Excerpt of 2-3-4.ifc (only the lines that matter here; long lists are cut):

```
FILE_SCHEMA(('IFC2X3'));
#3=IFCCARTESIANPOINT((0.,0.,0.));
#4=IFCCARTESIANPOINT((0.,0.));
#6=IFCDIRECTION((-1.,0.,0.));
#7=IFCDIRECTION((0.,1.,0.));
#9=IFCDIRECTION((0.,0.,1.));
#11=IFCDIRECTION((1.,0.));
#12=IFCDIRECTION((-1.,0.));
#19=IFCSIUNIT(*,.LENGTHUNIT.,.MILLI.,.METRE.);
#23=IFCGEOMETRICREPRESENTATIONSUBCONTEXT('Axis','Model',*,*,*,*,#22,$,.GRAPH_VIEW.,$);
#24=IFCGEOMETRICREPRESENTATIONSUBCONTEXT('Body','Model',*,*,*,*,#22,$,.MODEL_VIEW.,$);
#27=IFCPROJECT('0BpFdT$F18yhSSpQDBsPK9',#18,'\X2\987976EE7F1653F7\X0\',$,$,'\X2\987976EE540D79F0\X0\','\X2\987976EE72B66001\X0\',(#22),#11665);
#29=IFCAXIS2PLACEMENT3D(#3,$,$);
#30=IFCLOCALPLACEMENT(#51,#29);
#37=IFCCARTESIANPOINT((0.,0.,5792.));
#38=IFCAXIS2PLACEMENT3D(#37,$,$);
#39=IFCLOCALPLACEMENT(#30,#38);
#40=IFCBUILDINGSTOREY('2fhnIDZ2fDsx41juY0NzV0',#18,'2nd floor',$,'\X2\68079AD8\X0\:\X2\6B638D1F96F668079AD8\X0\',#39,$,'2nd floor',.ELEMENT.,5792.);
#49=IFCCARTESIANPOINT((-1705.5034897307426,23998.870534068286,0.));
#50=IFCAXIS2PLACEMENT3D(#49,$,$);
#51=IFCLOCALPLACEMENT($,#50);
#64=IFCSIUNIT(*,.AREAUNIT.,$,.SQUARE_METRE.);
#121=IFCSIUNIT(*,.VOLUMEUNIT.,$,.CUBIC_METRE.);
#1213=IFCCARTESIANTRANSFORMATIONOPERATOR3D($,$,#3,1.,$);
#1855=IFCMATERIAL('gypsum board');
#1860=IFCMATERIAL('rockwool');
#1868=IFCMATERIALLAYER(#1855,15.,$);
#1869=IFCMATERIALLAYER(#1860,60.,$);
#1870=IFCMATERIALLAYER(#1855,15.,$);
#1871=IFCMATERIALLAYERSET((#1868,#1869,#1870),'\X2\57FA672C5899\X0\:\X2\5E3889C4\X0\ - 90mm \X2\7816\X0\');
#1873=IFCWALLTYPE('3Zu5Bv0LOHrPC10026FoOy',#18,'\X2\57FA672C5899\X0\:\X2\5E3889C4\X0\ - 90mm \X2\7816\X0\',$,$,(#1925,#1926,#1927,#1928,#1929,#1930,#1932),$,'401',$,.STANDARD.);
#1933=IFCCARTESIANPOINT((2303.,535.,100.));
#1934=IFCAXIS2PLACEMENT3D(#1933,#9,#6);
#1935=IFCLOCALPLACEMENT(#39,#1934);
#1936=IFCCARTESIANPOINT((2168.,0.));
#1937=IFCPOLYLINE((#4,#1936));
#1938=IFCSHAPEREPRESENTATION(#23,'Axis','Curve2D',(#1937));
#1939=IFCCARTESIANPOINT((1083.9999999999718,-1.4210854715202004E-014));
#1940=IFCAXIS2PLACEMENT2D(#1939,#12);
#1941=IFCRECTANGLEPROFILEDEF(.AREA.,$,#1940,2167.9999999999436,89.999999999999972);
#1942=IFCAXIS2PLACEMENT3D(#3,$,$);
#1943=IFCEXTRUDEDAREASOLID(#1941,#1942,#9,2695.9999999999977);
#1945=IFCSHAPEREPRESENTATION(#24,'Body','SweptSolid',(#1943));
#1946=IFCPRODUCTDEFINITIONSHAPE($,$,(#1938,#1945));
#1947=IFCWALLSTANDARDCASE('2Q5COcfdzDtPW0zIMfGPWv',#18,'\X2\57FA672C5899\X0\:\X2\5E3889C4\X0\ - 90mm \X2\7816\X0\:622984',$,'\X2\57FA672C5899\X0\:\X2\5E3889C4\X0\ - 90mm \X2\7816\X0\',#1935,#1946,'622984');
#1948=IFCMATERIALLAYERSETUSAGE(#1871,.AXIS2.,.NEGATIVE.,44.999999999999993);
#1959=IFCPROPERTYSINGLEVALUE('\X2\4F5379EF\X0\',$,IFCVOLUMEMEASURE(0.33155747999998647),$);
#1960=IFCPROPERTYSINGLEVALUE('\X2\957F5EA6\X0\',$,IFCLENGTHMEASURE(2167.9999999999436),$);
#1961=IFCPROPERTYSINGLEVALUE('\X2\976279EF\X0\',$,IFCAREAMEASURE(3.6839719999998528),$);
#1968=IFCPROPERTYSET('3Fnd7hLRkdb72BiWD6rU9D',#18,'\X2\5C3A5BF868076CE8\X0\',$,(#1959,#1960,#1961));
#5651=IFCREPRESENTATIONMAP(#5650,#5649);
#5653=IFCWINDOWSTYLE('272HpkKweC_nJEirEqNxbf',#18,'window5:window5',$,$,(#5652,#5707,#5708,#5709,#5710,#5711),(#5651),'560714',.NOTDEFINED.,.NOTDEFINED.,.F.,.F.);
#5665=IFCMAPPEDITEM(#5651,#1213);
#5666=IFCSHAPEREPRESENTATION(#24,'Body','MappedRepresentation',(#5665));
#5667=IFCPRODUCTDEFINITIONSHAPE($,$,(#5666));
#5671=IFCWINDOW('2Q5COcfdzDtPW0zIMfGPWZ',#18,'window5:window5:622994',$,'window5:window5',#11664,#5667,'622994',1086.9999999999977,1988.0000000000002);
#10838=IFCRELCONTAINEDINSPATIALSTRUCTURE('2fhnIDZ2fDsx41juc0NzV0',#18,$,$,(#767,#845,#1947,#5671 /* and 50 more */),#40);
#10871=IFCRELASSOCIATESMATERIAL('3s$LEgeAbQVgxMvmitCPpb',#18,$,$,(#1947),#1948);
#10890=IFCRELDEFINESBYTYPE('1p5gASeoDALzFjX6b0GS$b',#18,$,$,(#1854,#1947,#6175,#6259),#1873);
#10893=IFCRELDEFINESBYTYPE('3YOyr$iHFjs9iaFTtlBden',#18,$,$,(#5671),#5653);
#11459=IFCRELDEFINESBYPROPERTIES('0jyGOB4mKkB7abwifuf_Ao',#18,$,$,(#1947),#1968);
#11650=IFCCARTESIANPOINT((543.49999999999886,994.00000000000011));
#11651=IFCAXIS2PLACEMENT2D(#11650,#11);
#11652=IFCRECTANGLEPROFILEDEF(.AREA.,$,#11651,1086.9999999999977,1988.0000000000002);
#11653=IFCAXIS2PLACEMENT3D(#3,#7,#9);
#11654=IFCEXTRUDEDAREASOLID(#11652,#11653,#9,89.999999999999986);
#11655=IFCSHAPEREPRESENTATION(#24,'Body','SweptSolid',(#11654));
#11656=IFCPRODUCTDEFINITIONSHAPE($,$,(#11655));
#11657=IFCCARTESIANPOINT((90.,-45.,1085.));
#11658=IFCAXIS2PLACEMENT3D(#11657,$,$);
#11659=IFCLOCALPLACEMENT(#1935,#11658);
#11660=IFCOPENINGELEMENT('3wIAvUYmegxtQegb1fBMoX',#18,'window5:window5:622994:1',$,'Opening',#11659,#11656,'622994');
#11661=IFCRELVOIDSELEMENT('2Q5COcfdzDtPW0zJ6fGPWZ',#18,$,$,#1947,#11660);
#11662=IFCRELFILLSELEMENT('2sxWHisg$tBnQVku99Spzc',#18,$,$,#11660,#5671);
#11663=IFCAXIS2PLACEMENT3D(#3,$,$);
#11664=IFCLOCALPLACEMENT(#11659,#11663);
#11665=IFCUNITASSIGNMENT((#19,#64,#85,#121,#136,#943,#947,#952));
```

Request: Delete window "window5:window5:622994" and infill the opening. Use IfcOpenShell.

```python
import ifcopenshell
import ifcopenshell.api.feature
import ifcopenshell.api.pset
import ifcopenshell.api.root
import ifcopenshell.geom
import ifcopenshell.util.element
import ifcopenshell.util.shape
import ifcopenshell.util.unit

model = ifcopenshell.open("2-3-4.ifc")
area_scale = ifcopenshell.util.unit.calculate_unit_scale(model, "AREAUNIT")
volume_scale = ifcopenshell.util.unit.calculate_unit_scale(model, "VOLUMEUNIT")
settings = ifcopenshell.geom.settings()


def volume(element):
    """Net volume in cubic metres, openings subtracted."""
    shape = ifcopenshell.geom.create_shape(settings, element)
    return ifcopenshell.util.shape.get_volume(shape.geometry)


window = model.by_guid("2Q5COcfdzDtPW0zIMfGPWZ")
opening = window.FillsVoids[0].RelatingOpeningElement
wall = opening.VoidsElements[0].RelatingBuildingElement
before = volume(wall)

ifcopenshell.api.root.remove_product(model, product=window)
ifcopenshell.api.feature.remove_feature(model, feature=opening)

after = volume(wall)
thickness = 0.09  # wall thickness in metres

# Update the wall's stored quantities.
pset = model.by_id(ifcopenshell.util.element.get_pset(wall, "尺寸标注", should_inherit=False)["id"])
ifcopenshell.api.pset.edit_pset(model, pset=pset, properties={
    "体积": model.create_entity("IfcVolumeMeasure", after / volume_scale),
    "面积": model.create_entity("IfcAreaMeasure", after / thickness / area_scale),
})

print(f"wall volume {before:.3f} -> {after:.3f} m3")

model.write("2-3-4-out.ifc")
```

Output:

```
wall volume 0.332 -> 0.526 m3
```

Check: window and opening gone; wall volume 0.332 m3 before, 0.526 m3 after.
